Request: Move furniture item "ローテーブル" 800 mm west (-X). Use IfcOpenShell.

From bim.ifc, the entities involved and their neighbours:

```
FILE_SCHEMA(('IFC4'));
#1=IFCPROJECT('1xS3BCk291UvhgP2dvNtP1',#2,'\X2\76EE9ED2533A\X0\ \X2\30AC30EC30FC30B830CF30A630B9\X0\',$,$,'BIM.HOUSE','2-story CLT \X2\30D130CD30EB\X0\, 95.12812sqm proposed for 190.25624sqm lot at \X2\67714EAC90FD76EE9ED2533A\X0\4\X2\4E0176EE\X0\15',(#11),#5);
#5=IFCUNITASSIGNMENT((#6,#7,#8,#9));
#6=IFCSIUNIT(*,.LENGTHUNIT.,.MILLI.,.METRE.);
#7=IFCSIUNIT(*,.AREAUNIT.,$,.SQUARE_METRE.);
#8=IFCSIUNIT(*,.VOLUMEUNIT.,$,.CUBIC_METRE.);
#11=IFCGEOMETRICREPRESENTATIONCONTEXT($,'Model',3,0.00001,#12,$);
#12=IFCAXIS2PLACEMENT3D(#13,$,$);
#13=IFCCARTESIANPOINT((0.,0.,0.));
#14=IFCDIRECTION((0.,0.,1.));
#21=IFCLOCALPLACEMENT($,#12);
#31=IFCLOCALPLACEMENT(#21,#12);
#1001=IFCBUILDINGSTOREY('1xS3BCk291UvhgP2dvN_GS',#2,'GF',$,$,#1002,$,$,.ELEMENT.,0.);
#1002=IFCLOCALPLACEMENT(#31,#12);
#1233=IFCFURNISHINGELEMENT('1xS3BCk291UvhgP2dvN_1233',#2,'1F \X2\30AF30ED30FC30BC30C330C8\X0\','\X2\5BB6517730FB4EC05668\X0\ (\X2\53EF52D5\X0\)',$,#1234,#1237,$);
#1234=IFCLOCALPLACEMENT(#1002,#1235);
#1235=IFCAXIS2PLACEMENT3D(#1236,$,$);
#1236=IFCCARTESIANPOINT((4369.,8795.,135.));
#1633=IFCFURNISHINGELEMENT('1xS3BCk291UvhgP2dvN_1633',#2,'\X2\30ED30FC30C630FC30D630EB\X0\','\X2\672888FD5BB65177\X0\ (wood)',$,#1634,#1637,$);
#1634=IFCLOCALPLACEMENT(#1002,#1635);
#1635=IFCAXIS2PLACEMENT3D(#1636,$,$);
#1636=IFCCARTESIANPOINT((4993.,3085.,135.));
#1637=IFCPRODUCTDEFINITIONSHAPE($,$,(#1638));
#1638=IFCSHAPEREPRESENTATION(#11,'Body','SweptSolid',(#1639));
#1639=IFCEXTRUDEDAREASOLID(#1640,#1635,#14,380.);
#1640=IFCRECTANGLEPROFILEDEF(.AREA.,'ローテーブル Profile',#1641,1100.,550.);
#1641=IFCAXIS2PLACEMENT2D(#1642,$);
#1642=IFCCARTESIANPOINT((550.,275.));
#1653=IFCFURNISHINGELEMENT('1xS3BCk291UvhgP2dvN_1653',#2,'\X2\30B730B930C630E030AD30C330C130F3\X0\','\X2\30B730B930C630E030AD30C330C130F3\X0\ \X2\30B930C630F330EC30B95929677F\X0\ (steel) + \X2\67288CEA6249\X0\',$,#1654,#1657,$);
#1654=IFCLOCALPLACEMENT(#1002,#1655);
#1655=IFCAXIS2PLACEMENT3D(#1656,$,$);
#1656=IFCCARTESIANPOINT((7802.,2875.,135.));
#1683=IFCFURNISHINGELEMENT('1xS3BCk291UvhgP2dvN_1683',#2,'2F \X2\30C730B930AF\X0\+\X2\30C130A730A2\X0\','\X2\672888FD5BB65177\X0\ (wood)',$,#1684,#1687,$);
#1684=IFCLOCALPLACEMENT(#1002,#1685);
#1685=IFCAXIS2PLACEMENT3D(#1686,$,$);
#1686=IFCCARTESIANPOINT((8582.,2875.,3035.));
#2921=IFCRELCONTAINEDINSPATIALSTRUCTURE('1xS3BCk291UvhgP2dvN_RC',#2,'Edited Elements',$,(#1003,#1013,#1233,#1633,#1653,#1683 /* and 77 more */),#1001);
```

```python
import ifcopenshell
import ifcopenshell.api.geometry
import ifcopenshell.util.placement

model = ifcopenshell.open("bim.ifc")

item = model.by_guid("1xS3BCk291UvhgP2dvN_1633")
matrix = ifcopenshell.util.placement.get_local_placement(item.ObjectPlacement)
matrix[0, 3] -= 800.0
ifcopenshell.api.geometry.edit_object_placement(model, product=item, matrix=matrix, is_si=False)

print(ifcopenshell.util.placement.get_local_placement(item.ObjectPlacement).round(3) + 0.0)

model.write("bim_v2.ifc")
```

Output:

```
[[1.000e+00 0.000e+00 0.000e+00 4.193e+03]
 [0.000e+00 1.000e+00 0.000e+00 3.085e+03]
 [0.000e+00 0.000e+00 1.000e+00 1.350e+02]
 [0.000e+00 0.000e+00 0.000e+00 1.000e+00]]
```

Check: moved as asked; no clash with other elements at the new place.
